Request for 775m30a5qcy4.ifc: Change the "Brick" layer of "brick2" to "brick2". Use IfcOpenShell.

First a look at what the model holds.

```python
import ifcopenshell
import ifcopenshell.util.element

model = ifcopenshell.open("775m30a5qcy4.ifc")
print(model.schema)
for layer_set in model.by_type("IfcMaterialLayerSet"):
    if layer_set.LayerSetName == "brick2":
        for layer in layer_set.MaterialLayers:
            print(layer.id(), layer.Material and layer.Material.Name, layer.LayerThickness, sep=" | ")
        print(len(ifcopenshell.util.element.get_elements_by_material(model, layer_set)), "elements and types use it")
print(sorted(m.Name for m in model.by_type("IfcMaterial") if m.Name)[:60])
```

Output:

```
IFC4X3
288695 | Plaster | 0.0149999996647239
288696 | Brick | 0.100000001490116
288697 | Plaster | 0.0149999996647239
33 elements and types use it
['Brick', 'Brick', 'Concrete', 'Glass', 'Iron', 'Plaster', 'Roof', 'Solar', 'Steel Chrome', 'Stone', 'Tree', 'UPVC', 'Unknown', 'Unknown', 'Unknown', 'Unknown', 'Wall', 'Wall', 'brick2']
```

```python
import ifcopenshell
import ifcopenshell.api.material

model = ifcopenshell.open("775m30a5qcy4.ifc")

layer_set = next(s for s in model.by_type("IfcMaterialLayerSet") if s.LayerSetName == "brick2")
layer = next(l for l in layer_set.MaterialLayers if l.Material and l.Material.Name == "Brick")
material = next(m for m in model.by_type("IfcMaterial") if m.Name == "brick2")

# Point this one layer at the other material; renaming the old one would change it everywhere.
ifcopenshell.api.material.edit_layer(model, layer=layer, attributes={}, material=material)

print([l.Material.Name if l.Material else None for l in layer_set.MaterialLayers])

model.write("775m30a5qcy4-out.ifc")
```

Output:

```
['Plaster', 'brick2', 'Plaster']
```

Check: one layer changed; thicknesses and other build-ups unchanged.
